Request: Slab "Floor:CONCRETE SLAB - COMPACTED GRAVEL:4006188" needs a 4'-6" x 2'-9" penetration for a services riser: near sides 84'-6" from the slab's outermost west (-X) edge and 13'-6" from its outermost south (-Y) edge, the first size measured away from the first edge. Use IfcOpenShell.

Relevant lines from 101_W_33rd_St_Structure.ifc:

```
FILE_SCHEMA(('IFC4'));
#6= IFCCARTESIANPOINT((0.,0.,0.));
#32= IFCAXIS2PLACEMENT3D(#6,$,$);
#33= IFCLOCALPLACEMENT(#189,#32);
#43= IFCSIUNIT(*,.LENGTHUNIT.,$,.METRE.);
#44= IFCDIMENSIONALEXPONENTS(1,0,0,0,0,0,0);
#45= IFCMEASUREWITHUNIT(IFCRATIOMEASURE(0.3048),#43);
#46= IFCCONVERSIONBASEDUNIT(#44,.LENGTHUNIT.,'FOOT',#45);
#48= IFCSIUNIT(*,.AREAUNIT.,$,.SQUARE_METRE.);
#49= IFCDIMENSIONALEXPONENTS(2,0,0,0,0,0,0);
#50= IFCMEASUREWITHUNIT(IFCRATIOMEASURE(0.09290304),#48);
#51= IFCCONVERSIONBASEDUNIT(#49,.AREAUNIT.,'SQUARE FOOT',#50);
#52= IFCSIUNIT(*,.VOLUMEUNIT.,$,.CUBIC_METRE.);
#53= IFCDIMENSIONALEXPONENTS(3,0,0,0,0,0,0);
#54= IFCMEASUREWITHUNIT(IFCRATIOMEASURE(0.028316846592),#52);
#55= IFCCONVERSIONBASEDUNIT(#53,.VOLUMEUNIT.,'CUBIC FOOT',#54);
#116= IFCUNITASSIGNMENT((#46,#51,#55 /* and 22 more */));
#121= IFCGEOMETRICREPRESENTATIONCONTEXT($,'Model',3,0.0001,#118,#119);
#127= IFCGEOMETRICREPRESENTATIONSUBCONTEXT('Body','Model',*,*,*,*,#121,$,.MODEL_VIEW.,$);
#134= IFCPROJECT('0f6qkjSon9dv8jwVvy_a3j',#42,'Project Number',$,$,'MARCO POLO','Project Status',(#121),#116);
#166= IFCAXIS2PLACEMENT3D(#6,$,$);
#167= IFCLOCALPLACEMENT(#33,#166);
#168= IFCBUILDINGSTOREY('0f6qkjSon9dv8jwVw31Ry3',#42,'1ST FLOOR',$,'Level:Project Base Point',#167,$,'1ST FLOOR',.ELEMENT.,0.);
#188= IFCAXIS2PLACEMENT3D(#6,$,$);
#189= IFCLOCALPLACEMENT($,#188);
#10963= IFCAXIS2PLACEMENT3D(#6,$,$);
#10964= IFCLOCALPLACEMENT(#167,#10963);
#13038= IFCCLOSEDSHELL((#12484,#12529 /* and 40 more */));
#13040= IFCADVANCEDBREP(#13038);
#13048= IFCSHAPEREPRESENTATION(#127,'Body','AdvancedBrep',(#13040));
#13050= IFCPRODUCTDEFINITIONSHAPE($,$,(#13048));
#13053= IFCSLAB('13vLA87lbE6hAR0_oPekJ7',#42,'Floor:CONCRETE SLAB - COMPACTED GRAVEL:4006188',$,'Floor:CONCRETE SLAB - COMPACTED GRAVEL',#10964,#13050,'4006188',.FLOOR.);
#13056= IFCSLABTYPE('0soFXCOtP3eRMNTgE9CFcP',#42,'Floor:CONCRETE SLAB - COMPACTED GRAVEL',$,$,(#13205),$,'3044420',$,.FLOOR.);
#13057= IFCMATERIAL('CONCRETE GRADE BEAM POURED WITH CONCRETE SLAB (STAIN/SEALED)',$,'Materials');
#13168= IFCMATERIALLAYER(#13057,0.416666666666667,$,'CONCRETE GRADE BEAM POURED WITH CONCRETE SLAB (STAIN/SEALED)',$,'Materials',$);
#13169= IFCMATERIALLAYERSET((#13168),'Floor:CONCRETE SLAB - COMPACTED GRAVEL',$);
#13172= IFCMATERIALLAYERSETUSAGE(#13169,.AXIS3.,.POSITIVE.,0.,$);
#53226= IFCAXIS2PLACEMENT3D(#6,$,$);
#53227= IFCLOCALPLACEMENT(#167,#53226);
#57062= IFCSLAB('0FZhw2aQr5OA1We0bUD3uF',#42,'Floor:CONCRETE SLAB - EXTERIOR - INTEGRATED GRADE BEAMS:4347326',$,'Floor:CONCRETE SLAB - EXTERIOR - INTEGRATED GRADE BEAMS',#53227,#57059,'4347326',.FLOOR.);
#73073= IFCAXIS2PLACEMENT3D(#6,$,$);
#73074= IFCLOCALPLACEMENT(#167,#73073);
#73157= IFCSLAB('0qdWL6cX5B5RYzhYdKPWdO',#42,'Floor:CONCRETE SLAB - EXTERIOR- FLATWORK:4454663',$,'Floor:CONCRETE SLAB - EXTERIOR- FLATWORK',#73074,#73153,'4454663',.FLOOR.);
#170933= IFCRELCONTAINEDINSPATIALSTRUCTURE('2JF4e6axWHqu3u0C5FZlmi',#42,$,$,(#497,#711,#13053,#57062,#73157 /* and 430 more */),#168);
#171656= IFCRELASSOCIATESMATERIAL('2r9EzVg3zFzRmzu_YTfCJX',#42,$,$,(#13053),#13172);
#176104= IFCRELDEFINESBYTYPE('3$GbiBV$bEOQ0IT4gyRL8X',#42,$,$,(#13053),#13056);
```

```python
import numpy as np
import ifcopenshell
import ifcopenshell.api.feature
import ifcopenshell.api.geometry
import ifcopenshell.api.root
import ifcopenshell.geom
import ifcopenshell.util.placement
import ifcopenshell.util.representation
import ifcopenshell.util.shape
import ifcopenshell.util.unit

model = ifcopenshell.open("101_W_33rd_St_Structure.ifc")
unit_scale = ifcopenshell.util.unit.calculate_unit_scale(model)
settings = ifcopenshell.geom.settings()


def volume(element):
    """Net volume in cubic metres, openings subtracted."""
    shape = ifcopenshell.geom.create_shape(settings, element)
    return ifcopenshell.util.shape.get_volume(shape.geometry)


slab = model.by_guid("13vLA87lbE6hAR0_oPekJ7")
before = volume(slab)

# Extent in the slab's own axes, in metres. The edges named are its -X and -Y sides.
slab_shape = ifcopenshell.geom.create_shape(settings, slab)
vertices = ifcopenshell.util.shape.get_vertices(slab_shape.geometry)
x_min, y_min, bottom = vertices.min(axis=0)
top = vertices[:, 2].max()

opening = ifcopenshell.api.root.create_entity(model, ifc_class="IfcOpeningElement", name="Services riser opening", predefined_type="OPENING")
context = ifcopenshell.util.representation.get_context(model, "Model", "Body", "MODEL_VIEW")
width, depth = 1.3716, 0.8382
outline = [(0.0, 0.0), (width, 0.0), (width, depth), (0.0, depth), (0.0, 0.0)]
# Overshoot both faces by 50 mm so the cut is clean.
shape = ifcopenshell.api.geometry.add_slab_representation(
    model, context=context, depth=top - bottom + 0.1, polyline=outline
)
ifcopenshell.api.geometry.assign_representation(model, product=opening, representation=shape)

matrix = ifcopenshell.util.placement.get_local_placement(slab.ObjectPlacement)
matrix[:, 3] = matrix @ np.append(np.array([x_min + 25.7556, y_min + 4.1148, bottom - 0.05]) / unit_scale, 1.0)
ifcopenshell.api.geometry.edit_object_placement(model, product=opening, matrix=matrix, is_si=False)
ifcopenshell.api.feature.add_feature(model, feature=opening, element=slab)

after = volume(slab)

print(f"slab volume {before:.3f} -> {after:.3f} m3")

model.write("101_W_33rd_St_Structure_edited.ifc")
```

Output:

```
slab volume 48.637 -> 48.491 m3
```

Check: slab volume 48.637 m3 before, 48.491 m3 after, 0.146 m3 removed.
